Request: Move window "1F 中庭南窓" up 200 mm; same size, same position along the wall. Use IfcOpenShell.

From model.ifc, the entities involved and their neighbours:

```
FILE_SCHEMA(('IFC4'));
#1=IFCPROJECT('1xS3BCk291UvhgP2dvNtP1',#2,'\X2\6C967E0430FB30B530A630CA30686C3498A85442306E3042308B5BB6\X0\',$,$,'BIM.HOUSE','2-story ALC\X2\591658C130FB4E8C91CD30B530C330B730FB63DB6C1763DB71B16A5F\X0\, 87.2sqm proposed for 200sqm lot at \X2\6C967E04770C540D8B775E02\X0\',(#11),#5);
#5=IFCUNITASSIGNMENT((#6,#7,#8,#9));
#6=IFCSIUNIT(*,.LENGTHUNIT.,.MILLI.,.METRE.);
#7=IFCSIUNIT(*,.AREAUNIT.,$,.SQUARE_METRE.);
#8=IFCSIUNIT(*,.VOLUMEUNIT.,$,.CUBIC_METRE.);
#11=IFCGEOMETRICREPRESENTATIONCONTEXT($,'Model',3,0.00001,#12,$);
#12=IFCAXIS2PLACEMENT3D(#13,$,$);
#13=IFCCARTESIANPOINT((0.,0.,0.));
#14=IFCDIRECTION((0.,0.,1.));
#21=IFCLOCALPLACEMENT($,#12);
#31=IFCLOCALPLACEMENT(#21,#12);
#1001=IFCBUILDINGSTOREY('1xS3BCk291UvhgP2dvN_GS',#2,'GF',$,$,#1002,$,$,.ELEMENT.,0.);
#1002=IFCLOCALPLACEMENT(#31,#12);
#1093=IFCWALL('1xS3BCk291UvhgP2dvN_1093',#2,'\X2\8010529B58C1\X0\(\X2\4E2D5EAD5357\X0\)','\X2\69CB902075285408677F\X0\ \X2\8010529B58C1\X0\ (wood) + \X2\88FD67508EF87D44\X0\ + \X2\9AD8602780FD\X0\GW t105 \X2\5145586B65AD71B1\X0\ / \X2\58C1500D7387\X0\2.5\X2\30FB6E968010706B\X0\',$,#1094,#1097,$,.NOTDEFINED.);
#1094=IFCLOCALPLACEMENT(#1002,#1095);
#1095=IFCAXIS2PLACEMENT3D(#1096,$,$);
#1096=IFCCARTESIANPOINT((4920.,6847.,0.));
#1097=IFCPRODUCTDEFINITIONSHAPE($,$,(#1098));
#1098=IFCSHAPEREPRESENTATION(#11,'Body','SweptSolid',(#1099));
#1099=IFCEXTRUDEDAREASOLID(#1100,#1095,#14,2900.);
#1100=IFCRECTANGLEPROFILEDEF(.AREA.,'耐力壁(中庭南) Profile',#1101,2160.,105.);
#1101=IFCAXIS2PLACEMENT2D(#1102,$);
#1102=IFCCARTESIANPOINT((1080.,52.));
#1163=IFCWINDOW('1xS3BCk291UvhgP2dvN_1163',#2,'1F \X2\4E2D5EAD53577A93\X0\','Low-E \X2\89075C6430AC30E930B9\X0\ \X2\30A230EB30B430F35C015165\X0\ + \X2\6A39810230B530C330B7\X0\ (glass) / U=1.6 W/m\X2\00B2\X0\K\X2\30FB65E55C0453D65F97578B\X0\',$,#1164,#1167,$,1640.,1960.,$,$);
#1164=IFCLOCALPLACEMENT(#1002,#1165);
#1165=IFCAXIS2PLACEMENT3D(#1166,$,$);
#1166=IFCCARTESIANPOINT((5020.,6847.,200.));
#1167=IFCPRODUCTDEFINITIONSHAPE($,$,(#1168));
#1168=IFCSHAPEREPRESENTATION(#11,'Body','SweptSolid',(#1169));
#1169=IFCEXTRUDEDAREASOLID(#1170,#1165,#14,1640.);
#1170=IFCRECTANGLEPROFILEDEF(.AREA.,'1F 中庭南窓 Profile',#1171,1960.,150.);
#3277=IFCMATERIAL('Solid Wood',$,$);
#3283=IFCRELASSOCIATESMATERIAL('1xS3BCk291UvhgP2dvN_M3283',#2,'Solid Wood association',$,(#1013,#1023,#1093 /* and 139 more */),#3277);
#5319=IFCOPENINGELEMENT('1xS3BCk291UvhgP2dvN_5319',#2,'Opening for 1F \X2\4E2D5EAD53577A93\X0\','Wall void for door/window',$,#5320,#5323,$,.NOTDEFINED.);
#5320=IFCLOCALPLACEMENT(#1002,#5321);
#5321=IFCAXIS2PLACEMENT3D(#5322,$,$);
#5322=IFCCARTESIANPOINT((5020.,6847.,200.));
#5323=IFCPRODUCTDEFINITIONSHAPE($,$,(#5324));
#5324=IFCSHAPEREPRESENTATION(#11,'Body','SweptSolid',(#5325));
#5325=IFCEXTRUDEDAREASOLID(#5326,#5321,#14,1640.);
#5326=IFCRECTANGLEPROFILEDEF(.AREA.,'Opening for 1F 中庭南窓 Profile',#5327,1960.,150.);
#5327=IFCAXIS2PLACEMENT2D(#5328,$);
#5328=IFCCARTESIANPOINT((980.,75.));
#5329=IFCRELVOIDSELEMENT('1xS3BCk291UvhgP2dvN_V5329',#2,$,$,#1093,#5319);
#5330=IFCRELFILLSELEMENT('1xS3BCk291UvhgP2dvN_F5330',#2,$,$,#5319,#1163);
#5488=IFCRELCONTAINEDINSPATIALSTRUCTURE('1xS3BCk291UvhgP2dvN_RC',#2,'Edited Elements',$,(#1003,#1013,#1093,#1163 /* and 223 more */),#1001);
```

```python
import numpy as np
import ifcopenshell
import ifcopenshell.api.geometry
import ifcopenshell.util.placement
import ifcopenshell.util.unit

model = ifcopenshell.open("model.ifc")
unit_scale = ifcopenshell.util.unit.calculate_unit_scale(model)

window = model.by_guid("1xS3BCk291UvhgP2dvN_1163")
opening = window.FillsVoids[0].RelatingOpeningElement
dz = 200.0

shift = np.array([0.0, 0.0, dz])
# The window is not placed relative to its opening, so move both.
for product in (opening, window):
    matrix = ifcopenshell.util.placement.get_local_placement(product.ObjectPlacement)
    matrix[:3, 3] += shift
    ifcopenshell.api.geometry.edit_object_placement(model, product=product, matrix=matrix, is_si=False)

print(f"moved by {dz * unit_scale:+.3f} m")

model.write("model_rev.ifc")
```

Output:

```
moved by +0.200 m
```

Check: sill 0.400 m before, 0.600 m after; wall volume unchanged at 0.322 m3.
